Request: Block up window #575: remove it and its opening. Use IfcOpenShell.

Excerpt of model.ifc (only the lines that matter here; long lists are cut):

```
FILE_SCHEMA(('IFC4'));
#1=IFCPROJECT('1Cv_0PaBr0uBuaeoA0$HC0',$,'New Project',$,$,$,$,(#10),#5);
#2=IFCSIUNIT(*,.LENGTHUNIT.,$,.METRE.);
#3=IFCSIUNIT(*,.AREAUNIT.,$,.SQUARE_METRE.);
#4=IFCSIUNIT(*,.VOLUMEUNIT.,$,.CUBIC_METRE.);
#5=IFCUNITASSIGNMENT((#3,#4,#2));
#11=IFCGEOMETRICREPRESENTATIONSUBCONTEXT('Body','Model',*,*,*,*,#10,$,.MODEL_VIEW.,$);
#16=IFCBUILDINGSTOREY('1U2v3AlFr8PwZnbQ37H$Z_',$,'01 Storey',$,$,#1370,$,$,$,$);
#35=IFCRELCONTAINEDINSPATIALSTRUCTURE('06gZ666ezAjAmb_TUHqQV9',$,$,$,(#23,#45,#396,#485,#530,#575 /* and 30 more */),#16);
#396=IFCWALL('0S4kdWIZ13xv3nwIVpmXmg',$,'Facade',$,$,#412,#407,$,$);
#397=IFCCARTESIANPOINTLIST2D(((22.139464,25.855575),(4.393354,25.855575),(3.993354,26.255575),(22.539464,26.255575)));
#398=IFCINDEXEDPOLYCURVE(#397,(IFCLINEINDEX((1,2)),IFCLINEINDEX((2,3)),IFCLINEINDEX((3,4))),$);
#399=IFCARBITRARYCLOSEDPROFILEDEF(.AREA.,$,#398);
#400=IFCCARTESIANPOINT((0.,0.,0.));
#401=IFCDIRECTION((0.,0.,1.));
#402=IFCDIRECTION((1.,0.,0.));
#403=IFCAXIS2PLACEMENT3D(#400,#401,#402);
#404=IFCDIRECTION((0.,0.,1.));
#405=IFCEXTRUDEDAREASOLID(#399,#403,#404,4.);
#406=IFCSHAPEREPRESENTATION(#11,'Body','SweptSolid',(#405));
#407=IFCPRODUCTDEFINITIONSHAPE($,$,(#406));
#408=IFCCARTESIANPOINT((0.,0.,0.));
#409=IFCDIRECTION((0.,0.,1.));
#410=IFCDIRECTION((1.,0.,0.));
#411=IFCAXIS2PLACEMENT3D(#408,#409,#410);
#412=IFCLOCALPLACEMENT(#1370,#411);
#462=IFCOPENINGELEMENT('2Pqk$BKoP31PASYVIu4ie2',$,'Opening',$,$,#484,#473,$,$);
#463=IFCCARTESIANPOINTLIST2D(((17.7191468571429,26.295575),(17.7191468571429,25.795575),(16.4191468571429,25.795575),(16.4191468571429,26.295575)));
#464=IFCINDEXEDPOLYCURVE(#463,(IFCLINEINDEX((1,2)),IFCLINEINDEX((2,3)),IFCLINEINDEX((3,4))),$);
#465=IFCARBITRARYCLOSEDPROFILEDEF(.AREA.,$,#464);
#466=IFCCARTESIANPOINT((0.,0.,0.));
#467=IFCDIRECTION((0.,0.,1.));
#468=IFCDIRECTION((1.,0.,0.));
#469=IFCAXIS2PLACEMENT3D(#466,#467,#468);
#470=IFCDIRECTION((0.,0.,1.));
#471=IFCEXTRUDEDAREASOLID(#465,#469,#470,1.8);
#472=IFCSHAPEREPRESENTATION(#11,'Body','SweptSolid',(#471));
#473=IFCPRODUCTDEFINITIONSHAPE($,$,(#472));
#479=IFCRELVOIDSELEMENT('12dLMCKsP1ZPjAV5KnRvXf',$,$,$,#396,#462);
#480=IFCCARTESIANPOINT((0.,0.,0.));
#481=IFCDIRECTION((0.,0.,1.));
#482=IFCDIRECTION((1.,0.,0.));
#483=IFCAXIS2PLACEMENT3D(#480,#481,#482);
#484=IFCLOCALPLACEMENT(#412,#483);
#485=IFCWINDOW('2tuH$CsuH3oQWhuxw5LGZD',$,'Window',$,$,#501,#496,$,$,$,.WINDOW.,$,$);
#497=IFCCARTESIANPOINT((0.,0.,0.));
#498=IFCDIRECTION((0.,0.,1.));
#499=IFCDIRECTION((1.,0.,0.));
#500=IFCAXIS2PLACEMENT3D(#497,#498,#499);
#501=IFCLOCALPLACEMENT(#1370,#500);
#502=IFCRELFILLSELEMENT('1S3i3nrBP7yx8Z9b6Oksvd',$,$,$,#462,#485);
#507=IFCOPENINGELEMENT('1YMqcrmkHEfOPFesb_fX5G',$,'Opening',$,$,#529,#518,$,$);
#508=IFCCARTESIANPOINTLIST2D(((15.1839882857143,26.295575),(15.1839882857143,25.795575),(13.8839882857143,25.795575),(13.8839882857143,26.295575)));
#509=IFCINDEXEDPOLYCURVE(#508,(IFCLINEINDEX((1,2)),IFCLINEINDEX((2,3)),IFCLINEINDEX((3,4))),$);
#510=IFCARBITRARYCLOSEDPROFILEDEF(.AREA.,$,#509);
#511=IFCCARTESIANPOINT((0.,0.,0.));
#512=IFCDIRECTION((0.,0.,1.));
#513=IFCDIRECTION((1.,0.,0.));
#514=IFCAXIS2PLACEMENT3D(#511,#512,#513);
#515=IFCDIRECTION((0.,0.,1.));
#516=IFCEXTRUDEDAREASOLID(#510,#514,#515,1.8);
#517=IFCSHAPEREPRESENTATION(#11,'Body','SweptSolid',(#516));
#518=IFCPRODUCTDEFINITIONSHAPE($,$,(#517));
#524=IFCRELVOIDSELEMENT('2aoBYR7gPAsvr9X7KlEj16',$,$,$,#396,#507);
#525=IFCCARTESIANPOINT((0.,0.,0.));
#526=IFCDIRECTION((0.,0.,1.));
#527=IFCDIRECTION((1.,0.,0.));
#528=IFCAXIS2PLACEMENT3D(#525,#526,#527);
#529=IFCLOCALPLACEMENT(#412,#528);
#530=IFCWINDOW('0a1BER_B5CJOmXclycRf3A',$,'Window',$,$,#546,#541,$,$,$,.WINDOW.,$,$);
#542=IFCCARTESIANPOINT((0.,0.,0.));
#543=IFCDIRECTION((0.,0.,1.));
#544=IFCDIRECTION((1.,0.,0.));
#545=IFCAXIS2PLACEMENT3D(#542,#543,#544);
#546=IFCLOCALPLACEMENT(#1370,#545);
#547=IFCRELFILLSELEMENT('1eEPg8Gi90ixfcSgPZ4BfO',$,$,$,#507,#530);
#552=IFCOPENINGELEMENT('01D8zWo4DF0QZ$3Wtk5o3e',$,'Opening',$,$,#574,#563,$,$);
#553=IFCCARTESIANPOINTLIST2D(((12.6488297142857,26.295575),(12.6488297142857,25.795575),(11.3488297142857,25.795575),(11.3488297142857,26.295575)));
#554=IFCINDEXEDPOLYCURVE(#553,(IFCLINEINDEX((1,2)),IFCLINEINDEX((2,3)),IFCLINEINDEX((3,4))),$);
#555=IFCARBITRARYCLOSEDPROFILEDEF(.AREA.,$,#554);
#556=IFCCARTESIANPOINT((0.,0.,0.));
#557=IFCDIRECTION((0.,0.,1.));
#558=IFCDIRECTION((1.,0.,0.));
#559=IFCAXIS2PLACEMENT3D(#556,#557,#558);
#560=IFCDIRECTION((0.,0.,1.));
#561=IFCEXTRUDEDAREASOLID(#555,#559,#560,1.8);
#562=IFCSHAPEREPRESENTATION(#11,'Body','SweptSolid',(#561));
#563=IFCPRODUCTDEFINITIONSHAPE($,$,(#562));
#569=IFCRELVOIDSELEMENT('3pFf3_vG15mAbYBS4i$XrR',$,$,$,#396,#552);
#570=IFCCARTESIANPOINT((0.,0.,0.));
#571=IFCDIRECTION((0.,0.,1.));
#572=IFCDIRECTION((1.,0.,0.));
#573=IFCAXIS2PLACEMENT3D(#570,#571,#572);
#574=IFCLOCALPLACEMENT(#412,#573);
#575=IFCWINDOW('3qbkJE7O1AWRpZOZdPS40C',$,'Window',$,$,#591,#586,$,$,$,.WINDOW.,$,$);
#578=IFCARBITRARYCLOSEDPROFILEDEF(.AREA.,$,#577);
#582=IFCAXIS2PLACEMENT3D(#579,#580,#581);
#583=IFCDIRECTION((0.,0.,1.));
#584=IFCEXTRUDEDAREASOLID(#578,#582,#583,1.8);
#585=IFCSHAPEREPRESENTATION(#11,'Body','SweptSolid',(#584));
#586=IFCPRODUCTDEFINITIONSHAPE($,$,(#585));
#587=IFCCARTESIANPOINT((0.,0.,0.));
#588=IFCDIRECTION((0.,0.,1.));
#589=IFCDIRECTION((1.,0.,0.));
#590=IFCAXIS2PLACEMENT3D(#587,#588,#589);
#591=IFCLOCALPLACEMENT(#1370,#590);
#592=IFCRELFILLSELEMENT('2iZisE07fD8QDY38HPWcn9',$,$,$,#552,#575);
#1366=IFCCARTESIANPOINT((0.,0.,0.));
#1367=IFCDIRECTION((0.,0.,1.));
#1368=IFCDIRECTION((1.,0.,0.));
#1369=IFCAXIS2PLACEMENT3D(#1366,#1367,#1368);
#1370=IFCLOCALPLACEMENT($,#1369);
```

```python
import ifcopenshell
import ifcopenshell.api.feature
import ifcopenshell.api.root
import ifcopenshell.geom
import ifcopenshell.util.shape

model = ifcopenshell.open("model.ifc")
settings = ifcopenshell.geom.settings()


def volume(element):
    """Net volume in cubic metres, openings subtracted."""
    shape = ifcopenshell.geom.create_shape(settings, element)
    return ifcopenshell.util.shape.get_volume(shape.geometry)


window = model.by_guid("3qbkJE7O1AWRpZOZdPS40C")
opening = window.FillsVoids[0].RelatingOpeningElement
wall = opening.VoidsElements[0].RelatingBuildingElement
before = volume(wall)

ifcopenshell.api.root.remove_product(model, product=window)
ifcopenshell.api.feature.remove_feature(model, feature=opening)

after = volume(wall)

print(f"wall volume {before:.3f} -> {after:.3f} m3")

model.write("model_rev.ifc")
```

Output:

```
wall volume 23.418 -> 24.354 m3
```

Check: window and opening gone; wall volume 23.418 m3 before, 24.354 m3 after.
